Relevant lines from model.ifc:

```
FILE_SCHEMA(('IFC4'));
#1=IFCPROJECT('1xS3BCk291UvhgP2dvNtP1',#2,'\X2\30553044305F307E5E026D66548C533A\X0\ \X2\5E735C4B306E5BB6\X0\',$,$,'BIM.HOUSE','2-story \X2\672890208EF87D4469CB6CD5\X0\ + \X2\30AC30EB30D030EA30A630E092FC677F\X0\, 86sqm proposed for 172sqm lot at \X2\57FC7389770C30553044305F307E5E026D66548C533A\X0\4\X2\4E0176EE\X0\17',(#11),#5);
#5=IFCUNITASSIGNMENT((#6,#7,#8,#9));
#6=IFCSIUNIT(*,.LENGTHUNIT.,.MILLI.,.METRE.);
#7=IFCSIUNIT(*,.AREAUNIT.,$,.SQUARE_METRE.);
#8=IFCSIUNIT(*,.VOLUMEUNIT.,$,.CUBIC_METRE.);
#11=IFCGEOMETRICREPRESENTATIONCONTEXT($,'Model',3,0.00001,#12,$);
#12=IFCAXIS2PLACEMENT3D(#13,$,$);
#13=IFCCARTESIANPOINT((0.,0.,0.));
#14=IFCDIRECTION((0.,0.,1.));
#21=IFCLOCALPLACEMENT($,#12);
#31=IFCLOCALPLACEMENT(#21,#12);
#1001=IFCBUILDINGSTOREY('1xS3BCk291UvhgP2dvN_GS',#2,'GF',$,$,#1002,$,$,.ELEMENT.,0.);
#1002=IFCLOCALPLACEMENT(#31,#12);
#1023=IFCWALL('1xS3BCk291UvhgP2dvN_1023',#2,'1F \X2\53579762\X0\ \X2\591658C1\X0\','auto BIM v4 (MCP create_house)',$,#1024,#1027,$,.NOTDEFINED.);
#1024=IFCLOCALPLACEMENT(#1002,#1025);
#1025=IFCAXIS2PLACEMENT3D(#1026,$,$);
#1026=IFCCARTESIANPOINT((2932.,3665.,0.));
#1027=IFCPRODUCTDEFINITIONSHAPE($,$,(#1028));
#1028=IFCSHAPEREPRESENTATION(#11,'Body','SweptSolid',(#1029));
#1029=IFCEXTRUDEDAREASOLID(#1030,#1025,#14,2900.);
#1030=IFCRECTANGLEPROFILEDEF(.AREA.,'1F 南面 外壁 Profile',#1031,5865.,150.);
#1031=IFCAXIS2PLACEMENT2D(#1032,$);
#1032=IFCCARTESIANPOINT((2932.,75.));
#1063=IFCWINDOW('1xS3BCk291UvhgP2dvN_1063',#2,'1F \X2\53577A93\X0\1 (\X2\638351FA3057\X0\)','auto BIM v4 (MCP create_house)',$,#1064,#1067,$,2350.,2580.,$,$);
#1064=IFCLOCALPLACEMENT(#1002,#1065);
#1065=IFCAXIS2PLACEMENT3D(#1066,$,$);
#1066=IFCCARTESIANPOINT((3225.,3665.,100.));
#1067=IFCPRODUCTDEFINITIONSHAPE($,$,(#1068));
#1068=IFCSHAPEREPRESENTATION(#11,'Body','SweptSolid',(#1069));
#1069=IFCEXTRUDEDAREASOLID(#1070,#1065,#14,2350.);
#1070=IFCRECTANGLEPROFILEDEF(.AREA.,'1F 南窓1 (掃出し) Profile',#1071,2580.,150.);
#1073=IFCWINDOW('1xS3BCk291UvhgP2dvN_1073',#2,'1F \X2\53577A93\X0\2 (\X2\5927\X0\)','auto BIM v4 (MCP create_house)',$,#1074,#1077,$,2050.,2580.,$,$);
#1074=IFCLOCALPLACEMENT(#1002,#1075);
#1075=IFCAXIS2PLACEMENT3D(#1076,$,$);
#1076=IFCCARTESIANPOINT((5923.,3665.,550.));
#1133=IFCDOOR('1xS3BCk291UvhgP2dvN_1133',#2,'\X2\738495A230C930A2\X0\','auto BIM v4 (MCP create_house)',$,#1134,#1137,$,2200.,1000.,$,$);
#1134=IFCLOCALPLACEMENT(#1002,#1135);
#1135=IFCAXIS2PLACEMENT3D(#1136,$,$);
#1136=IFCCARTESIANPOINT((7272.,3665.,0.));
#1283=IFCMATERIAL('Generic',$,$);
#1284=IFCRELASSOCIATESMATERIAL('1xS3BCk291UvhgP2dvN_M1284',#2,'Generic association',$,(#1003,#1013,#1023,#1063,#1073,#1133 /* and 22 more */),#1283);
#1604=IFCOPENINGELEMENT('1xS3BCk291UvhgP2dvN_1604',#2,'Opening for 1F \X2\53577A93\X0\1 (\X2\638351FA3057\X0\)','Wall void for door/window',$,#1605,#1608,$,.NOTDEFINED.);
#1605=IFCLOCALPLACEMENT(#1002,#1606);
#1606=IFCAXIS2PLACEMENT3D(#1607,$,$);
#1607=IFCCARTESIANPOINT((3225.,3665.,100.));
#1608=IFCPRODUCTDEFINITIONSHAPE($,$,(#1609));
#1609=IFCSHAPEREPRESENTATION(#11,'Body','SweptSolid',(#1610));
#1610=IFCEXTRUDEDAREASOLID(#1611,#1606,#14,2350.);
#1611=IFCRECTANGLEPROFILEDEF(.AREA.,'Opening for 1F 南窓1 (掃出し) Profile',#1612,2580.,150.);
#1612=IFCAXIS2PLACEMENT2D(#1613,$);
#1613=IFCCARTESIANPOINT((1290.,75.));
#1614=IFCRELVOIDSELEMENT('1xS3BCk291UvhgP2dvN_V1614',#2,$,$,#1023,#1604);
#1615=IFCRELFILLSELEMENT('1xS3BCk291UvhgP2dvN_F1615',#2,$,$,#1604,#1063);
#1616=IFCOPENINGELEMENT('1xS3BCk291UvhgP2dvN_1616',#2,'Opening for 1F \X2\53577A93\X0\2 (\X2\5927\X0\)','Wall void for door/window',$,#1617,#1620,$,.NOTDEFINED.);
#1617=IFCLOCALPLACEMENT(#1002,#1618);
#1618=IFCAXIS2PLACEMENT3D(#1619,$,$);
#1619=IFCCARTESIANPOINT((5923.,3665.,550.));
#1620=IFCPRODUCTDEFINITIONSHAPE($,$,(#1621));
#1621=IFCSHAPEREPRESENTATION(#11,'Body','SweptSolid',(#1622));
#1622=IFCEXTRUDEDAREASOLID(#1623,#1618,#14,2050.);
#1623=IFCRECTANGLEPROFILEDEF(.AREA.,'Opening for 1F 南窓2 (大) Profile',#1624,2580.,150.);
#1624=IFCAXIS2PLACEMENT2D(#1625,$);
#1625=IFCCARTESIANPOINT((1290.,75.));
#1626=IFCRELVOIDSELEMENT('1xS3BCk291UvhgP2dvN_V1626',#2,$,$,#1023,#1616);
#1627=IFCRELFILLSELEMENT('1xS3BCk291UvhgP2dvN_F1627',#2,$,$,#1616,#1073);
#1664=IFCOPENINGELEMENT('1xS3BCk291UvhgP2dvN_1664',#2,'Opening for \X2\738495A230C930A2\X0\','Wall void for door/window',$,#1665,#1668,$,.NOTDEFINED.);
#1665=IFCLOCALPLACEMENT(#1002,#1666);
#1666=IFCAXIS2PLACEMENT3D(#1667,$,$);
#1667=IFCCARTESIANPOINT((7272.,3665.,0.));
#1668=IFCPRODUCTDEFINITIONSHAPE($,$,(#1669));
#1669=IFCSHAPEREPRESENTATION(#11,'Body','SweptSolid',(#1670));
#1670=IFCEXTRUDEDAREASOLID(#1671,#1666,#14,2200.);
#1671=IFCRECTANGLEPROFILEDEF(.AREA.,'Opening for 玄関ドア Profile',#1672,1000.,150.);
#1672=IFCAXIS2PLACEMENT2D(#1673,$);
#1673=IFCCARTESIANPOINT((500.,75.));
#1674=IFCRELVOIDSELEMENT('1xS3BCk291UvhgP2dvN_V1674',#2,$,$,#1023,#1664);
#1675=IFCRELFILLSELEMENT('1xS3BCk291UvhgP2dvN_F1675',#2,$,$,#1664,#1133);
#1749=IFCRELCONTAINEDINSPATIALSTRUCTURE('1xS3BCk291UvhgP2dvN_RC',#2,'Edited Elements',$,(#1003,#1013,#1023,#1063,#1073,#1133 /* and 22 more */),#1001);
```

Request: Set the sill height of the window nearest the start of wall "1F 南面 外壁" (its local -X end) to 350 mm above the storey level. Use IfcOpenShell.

```python
import numpy as np
import ifcopenshell
import ifcopenshell.api.geometry
import ifcopenshell.geom
import ifcopenshell.util.element
import ifcopenshell.util.placement
import ifcopenshell.util.shape
import ifcopenshell.util.unit

model = ifcopenshell.open("model.ifc")
unit_scale = ifcopenshell.util.unit.calculate_unit_scale(model)

window = model.by_guid("1xS3BCk291UvhgP2dvN_1063")
opening = window.FillsVoids[0].RelatingOpeningElement
storey = ifcopenshell.util.element.get_container(window, ifc_class="IfcBuildingStorey")
level = ifcopenshell.util.placement.get_local_placement(storey.ObjectPlacement)[2, 3]

# The opening's origin need not be at the sill, so measure its lowest point.
shape = ifcopenshell.geom.create_shape(ifcopenshell.geom.settings(), opening)
bottom = ifcopenshell.util.shape.get_shape_bottom_elevation(shape, shape.geometry) / unit_scale
dz = level + 0.35 / unit_scale - bottom

shift = np.array([0.0, 0.0, dz])
# The window is not placed relative to its opening, so move both.
for product in (opening, window):
    matrix = ifcopenshell.util.placement.get_local_placement(product.ObjectPlacement)
    matrix[:3, 3] += shift
    ifcopenshell.api.geometry.edit_object_placement(model, product=product, matrix=matrix, is_si=False)

print(f"moved by {dz * unit_scale:+.3f} m")

model.write("model_rev.ifc")
```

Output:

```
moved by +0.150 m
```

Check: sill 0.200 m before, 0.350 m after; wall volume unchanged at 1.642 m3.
